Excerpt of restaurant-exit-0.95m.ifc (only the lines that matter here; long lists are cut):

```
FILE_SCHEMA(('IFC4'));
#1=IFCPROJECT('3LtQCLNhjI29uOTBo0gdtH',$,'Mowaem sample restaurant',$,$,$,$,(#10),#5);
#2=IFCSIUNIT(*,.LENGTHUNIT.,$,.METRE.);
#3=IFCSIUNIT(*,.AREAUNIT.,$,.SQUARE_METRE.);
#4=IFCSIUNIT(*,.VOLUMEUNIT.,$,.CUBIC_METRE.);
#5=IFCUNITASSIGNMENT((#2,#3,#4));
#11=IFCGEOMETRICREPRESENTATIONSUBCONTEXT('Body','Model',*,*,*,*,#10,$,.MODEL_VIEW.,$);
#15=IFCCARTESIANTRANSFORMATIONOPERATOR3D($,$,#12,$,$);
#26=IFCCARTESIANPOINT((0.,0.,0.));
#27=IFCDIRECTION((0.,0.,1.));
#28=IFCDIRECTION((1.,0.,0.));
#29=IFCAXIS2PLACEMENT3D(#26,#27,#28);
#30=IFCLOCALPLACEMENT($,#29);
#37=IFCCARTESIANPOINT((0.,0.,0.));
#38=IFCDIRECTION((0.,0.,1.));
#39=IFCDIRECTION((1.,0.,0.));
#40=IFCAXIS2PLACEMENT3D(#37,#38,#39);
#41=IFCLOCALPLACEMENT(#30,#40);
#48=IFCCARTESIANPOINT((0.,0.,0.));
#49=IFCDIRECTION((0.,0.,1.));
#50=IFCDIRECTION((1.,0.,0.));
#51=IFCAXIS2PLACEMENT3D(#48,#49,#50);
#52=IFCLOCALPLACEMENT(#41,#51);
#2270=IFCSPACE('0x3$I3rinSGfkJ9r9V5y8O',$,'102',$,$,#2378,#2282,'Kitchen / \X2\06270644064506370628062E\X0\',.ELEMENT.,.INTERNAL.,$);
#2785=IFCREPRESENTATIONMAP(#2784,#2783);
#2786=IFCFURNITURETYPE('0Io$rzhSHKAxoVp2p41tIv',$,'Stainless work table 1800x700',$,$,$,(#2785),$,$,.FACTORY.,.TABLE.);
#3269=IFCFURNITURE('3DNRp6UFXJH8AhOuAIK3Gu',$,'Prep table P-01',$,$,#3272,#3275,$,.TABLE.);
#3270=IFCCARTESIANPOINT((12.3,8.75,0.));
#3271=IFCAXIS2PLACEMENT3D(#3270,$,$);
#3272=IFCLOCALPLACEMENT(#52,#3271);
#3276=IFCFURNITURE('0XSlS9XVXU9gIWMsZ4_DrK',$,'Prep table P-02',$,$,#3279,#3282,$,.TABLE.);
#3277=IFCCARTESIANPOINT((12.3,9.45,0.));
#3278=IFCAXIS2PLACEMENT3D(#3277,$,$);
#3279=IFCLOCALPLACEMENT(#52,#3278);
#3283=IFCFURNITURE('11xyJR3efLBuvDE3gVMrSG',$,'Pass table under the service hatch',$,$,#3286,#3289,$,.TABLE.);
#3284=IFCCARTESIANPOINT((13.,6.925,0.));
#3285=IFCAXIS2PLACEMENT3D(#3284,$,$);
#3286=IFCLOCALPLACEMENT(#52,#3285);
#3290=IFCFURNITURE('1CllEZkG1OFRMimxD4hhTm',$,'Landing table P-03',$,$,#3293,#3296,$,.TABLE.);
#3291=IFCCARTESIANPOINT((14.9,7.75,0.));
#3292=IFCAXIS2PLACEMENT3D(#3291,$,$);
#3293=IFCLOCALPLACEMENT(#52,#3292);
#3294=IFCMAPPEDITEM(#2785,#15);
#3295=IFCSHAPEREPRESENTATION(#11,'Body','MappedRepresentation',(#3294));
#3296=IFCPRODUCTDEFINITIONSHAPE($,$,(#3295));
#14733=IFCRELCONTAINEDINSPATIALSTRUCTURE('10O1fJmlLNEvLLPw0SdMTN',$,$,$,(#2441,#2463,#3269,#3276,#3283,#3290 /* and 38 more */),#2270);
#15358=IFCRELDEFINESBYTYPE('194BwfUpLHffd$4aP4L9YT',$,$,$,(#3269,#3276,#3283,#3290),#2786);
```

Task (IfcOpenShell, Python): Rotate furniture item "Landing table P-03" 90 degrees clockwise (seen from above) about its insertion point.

```python
import ifcopenshell
import ifcopenshell.api.geometry
import ifcopenshell.util.placement

model = ifcopenshell.open("restaurant-exit-0.95m.ifc")

item = model.by_guid("1CllEZkG1OFRMimxD4hhTm")
matrix = ifcopenshell.util.placement.get_local_placement(item.ObjectPlacement)
matrix = matrix @ ifcopenshell.util.placement.rotation(-90, "Z")
ifcopenshell.api.geometry.edit_object_placement(model, product=item, matrix=matrix, is_si=False)

print(ifcopenshell.util.placement.get_local_placement(item.ObjectPlacement).round(3) + 0.0)

model.write("restaurant-exit-0.95m-out.ifc")
```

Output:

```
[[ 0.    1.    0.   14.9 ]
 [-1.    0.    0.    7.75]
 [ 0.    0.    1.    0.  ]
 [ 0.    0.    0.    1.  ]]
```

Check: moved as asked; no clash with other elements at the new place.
